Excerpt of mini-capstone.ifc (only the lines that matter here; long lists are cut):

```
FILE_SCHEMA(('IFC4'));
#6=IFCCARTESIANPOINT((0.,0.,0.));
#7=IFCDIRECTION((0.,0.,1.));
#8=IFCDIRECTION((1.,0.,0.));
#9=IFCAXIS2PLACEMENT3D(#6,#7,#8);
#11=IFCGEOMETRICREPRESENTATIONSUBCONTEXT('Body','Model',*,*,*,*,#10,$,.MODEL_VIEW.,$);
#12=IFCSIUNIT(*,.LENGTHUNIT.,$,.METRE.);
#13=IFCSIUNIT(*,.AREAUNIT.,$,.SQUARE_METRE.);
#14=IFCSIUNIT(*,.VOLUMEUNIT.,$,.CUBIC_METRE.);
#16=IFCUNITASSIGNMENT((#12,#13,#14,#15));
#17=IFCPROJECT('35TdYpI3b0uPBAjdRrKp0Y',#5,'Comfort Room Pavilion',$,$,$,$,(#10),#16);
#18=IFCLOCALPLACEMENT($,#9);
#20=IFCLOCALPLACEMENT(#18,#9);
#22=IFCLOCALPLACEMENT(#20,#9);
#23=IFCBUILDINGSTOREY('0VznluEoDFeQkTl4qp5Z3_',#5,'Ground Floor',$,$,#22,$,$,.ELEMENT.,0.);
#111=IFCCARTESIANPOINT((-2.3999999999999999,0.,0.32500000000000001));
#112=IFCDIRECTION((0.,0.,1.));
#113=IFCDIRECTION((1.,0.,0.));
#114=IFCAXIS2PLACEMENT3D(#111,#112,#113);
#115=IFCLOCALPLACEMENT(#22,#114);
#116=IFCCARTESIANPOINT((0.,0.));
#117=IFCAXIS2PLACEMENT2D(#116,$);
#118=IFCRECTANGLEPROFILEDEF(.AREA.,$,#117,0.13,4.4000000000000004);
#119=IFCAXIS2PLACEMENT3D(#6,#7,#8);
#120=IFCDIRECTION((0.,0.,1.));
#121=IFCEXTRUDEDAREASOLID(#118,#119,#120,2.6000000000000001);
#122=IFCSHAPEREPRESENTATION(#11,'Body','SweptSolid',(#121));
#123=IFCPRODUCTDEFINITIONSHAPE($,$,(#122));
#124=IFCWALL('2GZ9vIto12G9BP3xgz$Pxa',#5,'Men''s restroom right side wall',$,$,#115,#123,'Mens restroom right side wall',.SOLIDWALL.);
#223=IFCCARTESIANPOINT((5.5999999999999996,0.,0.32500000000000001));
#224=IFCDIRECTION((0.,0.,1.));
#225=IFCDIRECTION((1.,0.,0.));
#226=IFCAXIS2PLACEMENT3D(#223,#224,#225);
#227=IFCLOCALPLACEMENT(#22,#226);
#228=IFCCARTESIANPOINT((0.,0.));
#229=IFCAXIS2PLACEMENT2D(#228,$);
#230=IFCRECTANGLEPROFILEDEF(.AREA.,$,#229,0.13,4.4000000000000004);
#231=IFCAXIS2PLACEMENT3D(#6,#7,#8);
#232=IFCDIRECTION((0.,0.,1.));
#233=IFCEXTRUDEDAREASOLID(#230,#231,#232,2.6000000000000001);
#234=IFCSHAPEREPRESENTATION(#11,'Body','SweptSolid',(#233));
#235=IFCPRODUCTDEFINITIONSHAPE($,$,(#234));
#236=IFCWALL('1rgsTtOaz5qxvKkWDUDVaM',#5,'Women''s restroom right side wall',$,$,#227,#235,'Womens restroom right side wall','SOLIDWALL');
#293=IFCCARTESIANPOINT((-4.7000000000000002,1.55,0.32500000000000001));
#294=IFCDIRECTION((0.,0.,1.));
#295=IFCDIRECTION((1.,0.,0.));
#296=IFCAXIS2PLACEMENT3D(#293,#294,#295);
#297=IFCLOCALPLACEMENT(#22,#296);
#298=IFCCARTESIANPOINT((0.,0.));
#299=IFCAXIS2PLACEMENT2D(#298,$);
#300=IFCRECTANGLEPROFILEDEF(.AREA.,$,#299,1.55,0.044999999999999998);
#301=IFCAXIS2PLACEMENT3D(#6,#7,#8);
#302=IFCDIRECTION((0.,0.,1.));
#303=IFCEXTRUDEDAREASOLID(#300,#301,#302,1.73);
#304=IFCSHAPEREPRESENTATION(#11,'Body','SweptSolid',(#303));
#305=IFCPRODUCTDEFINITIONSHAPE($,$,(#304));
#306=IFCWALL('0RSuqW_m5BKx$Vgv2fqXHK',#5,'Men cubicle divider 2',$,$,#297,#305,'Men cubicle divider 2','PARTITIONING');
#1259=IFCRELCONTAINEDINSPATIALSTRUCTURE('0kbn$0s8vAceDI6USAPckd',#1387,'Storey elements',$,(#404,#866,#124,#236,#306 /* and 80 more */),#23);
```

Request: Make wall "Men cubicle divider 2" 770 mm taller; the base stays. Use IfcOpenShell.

```python
import ifcopenshell
import ifcopenshell.geom
import ifcopenshell.util.representation
import ifcopenshell.util.shape

model = ifcopenshell.open("mini-capstone.ifc")
settings = ifcopenshell.geom.settings()


def volume(element):
    """Net volume in cubic metres, openings subtracted."""
    shape = ifcopenshell.geom.create_shape(settings, element)
    return ifcopenshell.util.shape.get_volume(shape.geometry)


wall = model.by_id(306)
before = volume(wall)

body = ifcopenshell.util.representation.get_representation(wall, "Model", "Body")
solid = body.Items[0]
old_height = solid.Depth
solid.Depth += 0.77
after = volume(wall)

print(f"height {old_height:g} -> {solid.Depth:g}, volume {before:.3f} -> {after:.3f} m3")

model.write("mini-capstone_rev.ifc")
```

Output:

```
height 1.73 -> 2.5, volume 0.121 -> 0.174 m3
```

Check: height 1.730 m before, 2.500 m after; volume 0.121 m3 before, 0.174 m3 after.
